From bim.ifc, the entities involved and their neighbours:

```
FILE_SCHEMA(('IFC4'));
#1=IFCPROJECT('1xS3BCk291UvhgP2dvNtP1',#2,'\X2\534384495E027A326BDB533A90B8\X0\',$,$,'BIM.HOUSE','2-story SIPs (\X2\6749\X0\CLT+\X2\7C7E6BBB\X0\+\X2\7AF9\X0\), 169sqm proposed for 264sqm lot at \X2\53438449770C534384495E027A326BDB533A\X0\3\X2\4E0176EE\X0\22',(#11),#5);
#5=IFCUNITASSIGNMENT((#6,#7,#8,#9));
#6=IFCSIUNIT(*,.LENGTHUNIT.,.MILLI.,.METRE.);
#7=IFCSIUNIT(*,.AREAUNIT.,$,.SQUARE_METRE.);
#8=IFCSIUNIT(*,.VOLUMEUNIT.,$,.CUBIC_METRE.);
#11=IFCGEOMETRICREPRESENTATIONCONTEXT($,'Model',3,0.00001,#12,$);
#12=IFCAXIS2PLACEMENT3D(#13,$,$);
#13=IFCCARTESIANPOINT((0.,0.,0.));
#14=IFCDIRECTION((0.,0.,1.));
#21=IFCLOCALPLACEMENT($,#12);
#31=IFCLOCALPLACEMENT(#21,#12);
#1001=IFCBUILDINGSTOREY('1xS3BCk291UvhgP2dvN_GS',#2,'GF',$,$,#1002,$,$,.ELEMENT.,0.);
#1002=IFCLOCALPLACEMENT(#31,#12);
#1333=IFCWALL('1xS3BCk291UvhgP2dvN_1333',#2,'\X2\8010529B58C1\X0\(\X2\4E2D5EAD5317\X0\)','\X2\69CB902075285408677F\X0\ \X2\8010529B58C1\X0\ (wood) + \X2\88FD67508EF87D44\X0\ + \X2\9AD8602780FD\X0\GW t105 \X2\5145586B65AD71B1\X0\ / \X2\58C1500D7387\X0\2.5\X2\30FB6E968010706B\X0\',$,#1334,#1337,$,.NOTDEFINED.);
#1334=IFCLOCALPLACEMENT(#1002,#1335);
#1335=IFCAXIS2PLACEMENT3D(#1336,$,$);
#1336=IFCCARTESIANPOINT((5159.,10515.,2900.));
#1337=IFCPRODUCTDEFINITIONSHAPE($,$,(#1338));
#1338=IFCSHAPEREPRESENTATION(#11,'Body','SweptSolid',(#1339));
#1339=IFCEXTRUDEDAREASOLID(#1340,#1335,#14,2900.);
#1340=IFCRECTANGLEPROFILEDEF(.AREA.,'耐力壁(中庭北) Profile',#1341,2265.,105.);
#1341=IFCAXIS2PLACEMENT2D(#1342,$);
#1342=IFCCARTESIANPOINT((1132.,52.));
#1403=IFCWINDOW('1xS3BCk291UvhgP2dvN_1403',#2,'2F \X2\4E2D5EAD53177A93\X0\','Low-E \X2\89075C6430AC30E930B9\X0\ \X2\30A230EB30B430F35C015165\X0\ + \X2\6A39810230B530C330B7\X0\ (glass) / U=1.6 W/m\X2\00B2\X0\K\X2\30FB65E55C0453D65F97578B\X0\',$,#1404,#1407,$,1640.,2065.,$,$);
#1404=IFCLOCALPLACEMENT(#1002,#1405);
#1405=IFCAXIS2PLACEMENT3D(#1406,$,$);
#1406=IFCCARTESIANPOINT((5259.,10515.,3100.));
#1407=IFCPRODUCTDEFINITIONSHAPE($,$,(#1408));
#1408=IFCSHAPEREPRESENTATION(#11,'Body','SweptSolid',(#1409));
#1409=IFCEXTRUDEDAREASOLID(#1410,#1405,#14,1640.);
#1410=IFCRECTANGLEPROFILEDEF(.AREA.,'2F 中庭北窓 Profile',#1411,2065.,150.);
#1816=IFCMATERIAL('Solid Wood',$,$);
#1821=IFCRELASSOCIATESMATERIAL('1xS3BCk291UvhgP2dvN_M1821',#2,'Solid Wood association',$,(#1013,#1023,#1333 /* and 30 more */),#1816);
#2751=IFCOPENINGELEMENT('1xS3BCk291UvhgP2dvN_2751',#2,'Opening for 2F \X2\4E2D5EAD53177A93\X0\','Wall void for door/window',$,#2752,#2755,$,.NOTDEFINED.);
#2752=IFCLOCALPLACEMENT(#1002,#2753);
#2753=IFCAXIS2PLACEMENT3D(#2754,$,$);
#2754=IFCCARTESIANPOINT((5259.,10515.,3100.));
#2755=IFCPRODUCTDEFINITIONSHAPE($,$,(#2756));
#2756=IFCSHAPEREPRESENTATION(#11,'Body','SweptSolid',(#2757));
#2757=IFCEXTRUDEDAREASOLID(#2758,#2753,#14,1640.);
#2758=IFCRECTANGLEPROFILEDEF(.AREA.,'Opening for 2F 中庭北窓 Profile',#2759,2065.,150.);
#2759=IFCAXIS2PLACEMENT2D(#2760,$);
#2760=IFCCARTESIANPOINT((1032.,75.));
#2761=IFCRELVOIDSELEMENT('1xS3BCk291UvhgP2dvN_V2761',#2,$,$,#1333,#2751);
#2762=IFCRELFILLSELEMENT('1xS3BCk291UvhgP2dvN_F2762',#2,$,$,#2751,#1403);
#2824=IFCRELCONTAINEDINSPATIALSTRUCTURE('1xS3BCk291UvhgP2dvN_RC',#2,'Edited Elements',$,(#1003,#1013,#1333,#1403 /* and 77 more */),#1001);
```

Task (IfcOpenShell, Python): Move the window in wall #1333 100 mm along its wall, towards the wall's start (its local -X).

```python
import ifcopenshell
import ifcopenshell.api.geometry
import ifcopenshell.util.placement
import ifcopenshell.util.unit

model = ifcopenshell.open("bim.ifc")
unit_scale = ifcopenshell.util.unit.calculate_unit_scale(model)

window = model.by_guid("1xS3BCk291UvhgP2dvN_1403")
opening = window.FillsVoids[0].RelatingOpeningElement
wall = opening.VoidsElements[0].RelatingBuildingElement

wall_matrix = ifcopenshell.util.placement.get_local_placement(wall.ObjectPlacement)
shift = wall_matrix[:3, 0] * -0.1 / unit_scale
before = ifcopenshell.util.placement.get_local_placement(window.ObjectPlacement)[:3, 3].copy()

# The window is not placed relative to its opening, so move both.
for product in (opening, window):
    matrix = ifcopenshell.util.placement.get_local_placement(product.ObjectPlacement)
    matrix[:3, 3] += shift
    ifcopenshell.api.geometry.edit_object_placement(model, product=product, matrix=matrix, is_si=False)

after = ifcopenshell.util.placement.get_local_placement(window.ObjectPlacement)[:3, 3]
print("window moved by", (after - before).round(3) + 0.0)

model.write("bim_v2.ifc")
```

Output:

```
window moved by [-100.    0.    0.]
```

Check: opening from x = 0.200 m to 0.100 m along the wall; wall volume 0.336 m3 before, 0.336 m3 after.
